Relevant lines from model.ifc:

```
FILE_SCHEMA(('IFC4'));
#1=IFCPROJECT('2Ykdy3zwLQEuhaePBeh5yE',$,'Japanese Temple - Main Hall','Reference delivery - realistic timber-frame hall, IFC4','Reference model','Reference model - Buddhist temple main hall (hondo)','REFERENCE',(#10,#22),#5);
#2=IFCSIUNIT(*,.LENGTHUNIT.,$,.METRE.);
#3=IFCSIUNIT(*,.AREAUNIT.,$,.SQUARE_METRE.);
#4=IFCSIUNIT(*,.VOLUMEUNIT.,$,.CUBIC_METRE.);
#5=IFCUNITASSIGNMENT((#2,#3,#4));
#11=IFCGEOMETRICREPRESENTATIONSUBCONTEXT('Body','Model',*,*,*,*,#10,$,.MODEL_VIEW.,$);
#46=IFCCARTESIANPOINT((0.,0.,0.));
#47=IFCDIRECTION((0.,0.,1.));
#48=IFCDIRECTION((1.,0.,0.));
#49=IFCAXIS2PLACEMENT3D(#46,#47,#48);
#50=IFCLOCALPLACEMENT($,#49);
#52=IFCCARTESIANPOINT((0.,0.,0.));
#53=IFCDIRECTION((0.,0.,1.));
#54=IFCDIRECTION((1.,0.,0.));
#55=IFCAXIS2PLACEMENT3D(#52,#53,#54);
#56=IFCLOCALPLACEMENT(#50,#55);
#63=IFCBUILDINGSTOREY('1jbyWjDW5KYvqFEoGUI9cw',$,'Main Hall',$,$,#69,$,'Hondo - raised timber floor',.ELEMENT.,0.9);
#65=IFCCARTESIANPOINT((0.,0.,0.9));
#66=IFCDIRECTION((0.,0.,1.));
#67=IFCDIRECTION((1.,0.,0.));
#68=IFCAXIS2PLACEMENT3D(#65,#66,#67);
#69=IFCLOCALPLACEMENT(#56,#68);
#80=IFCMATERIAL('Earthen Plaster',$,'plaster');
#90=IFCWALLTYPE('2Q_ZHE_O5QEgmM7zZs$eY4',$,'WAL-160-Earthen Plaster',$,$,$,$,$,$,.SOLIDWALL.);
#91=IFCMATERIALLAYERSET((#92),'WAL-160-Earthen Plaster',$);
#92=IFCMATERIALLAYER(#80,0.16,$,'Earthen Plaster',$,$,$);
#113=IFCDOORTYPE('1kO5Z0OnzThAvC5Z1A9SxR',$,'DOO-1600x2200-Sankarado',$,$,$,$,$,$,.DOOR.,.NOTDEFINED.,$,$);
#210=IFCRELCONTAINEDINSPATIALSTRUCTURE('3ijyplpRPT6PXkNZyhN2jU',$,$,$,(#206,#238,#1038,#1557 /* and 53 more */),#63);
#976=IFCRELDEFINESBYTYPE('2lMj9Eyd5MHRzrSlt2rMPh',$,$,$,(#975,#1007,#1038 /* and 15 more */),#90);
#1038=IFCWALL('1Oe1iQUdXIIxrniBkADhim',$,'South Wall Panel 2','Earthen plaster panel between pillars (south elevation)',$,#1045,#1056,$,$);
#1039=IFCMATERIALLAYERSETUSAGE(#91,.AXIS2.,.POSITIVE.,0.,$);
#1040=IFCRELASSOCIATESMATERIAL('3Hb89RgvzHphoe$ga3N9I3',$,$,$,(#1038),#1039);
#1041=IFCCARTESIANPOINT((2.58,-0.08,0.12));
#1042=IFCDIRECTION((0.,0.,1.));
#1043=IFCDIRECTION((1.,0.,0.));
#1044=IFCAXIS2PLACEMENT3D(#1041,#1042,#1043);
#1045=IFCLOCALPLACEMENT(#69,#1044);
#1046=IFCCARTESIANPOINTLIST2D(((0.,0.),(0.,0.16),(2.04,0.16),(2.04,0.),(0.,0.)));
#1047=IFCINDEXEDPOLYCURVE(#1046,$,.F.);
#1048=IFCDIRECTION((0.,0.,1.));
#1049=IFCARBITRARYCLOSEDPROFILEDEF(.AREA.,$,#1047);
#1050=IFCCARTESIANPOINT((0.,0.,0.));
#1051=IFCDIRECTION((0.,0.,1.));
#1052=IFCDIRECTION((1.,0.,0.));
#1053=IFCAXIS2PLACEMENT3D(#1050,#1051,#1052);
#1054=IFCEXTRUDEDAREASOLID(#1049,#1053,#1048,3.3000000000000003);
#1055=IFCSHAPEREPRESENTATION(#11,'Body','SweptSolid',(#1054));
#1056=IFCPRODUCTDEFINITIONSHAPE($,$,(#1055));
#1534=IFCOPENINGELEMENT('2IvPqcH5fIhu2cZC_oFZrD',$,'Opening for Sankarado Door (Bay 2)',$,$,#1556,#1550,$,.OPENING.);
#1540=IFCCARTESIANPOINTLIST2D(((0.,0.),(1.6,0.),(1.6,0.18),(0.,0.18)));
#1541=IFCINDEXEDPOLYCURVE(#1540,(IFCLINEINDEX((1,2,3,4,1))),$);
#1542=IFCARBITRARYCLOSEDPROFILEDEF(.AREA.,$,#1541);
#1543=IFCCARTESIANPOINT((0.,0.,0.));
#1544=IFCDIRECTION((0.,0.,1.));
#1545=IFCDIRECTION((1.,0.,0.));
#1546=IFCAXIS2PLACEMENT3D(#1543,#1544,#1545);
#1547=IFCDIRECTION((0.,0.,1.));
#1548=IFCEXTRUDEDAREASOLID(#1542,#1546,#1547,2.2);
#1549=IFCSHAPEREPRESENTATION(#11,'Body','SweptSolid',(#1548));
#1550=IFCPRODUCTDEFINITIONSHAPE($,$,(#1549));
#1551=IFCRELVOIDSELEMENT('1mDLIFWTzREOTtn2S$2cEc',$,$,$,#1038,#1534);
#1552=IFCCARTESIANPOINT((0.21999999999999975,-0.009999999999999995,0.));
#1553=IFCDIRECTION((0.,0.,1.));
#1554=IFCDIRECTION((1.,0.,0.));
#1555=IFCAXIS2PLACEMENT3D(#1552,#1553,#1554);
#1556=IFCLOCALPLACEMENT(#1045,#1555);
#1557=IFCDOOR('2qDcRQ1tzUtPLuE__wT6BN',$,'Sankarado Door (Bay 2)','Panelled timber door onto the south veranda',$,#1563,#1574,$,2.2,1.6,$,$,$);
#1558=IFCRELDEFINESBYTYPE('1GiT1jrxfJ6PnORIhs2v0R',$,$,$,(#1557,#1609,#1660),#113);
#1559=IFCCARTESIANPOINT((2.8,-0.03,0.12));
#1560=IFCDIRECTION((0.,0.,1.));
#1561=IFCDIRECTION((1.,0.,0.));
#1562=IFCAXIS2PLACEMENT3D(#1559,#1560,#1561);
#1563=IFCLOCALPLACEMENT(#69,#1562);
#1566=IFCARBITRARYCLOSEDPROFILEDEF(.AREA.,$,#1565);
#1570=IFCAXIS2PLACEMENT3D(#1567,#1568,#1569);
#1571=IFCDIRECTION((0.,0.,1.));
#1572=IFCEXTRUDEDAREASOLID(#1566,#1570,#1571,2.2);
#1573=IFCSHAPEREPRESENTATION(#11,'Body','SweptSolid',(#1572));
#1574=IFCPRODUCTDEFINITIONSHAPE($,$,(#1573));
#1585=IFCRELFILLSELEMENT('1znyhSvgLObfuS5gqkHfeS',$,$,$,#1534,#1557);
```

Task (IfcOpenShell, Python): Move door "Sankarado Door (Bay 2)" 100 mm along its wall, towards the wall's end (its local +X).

```python
import ifcopenshell
import ifcopenshell.api.geometry
import ifcopenshell.util.placement

model = ifcopenshell.open("model.ifc")

door = model.by_guid("2qDcRQ1tzUtPLuE__wT6BN")
opening = door.FillsVoids[0].RelatingOpeningElement
wall = opening.VoidsElements[0].RelatingBuildingElement

wall_matrix = ifcopenshell.util.placement.get_local_placement(wall.ObjectPlacement)
shift = wall_matrix[:3, 0] * 0.1
before = ifcopenshell.util.placement.get_local_placement(door.ObjectPlacement)[:3, 3].copy()

# The door is not placed relative to its opening, so move both.
for product in (opening, door):
    matrix = ifcopenshell.util.placement.get_local_placement(product.ObjectPlacement)
    matrix[:3, 3] += shift
    ifcopenshell.api.geometry.edit_object_placement(model, product=product, matrix=matrix, is_si=False)

after = ifcopenshell.util.placement.get_local_placement(door.ObjectPlacement)[:3, 3]
print("door moved by", (after - before).round(3) + 0.0)

model.write("model_v2.ifc")
```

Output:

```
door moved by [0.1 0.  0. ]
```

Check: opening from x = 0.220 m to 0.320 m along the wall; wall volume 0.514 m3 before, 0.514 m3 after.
